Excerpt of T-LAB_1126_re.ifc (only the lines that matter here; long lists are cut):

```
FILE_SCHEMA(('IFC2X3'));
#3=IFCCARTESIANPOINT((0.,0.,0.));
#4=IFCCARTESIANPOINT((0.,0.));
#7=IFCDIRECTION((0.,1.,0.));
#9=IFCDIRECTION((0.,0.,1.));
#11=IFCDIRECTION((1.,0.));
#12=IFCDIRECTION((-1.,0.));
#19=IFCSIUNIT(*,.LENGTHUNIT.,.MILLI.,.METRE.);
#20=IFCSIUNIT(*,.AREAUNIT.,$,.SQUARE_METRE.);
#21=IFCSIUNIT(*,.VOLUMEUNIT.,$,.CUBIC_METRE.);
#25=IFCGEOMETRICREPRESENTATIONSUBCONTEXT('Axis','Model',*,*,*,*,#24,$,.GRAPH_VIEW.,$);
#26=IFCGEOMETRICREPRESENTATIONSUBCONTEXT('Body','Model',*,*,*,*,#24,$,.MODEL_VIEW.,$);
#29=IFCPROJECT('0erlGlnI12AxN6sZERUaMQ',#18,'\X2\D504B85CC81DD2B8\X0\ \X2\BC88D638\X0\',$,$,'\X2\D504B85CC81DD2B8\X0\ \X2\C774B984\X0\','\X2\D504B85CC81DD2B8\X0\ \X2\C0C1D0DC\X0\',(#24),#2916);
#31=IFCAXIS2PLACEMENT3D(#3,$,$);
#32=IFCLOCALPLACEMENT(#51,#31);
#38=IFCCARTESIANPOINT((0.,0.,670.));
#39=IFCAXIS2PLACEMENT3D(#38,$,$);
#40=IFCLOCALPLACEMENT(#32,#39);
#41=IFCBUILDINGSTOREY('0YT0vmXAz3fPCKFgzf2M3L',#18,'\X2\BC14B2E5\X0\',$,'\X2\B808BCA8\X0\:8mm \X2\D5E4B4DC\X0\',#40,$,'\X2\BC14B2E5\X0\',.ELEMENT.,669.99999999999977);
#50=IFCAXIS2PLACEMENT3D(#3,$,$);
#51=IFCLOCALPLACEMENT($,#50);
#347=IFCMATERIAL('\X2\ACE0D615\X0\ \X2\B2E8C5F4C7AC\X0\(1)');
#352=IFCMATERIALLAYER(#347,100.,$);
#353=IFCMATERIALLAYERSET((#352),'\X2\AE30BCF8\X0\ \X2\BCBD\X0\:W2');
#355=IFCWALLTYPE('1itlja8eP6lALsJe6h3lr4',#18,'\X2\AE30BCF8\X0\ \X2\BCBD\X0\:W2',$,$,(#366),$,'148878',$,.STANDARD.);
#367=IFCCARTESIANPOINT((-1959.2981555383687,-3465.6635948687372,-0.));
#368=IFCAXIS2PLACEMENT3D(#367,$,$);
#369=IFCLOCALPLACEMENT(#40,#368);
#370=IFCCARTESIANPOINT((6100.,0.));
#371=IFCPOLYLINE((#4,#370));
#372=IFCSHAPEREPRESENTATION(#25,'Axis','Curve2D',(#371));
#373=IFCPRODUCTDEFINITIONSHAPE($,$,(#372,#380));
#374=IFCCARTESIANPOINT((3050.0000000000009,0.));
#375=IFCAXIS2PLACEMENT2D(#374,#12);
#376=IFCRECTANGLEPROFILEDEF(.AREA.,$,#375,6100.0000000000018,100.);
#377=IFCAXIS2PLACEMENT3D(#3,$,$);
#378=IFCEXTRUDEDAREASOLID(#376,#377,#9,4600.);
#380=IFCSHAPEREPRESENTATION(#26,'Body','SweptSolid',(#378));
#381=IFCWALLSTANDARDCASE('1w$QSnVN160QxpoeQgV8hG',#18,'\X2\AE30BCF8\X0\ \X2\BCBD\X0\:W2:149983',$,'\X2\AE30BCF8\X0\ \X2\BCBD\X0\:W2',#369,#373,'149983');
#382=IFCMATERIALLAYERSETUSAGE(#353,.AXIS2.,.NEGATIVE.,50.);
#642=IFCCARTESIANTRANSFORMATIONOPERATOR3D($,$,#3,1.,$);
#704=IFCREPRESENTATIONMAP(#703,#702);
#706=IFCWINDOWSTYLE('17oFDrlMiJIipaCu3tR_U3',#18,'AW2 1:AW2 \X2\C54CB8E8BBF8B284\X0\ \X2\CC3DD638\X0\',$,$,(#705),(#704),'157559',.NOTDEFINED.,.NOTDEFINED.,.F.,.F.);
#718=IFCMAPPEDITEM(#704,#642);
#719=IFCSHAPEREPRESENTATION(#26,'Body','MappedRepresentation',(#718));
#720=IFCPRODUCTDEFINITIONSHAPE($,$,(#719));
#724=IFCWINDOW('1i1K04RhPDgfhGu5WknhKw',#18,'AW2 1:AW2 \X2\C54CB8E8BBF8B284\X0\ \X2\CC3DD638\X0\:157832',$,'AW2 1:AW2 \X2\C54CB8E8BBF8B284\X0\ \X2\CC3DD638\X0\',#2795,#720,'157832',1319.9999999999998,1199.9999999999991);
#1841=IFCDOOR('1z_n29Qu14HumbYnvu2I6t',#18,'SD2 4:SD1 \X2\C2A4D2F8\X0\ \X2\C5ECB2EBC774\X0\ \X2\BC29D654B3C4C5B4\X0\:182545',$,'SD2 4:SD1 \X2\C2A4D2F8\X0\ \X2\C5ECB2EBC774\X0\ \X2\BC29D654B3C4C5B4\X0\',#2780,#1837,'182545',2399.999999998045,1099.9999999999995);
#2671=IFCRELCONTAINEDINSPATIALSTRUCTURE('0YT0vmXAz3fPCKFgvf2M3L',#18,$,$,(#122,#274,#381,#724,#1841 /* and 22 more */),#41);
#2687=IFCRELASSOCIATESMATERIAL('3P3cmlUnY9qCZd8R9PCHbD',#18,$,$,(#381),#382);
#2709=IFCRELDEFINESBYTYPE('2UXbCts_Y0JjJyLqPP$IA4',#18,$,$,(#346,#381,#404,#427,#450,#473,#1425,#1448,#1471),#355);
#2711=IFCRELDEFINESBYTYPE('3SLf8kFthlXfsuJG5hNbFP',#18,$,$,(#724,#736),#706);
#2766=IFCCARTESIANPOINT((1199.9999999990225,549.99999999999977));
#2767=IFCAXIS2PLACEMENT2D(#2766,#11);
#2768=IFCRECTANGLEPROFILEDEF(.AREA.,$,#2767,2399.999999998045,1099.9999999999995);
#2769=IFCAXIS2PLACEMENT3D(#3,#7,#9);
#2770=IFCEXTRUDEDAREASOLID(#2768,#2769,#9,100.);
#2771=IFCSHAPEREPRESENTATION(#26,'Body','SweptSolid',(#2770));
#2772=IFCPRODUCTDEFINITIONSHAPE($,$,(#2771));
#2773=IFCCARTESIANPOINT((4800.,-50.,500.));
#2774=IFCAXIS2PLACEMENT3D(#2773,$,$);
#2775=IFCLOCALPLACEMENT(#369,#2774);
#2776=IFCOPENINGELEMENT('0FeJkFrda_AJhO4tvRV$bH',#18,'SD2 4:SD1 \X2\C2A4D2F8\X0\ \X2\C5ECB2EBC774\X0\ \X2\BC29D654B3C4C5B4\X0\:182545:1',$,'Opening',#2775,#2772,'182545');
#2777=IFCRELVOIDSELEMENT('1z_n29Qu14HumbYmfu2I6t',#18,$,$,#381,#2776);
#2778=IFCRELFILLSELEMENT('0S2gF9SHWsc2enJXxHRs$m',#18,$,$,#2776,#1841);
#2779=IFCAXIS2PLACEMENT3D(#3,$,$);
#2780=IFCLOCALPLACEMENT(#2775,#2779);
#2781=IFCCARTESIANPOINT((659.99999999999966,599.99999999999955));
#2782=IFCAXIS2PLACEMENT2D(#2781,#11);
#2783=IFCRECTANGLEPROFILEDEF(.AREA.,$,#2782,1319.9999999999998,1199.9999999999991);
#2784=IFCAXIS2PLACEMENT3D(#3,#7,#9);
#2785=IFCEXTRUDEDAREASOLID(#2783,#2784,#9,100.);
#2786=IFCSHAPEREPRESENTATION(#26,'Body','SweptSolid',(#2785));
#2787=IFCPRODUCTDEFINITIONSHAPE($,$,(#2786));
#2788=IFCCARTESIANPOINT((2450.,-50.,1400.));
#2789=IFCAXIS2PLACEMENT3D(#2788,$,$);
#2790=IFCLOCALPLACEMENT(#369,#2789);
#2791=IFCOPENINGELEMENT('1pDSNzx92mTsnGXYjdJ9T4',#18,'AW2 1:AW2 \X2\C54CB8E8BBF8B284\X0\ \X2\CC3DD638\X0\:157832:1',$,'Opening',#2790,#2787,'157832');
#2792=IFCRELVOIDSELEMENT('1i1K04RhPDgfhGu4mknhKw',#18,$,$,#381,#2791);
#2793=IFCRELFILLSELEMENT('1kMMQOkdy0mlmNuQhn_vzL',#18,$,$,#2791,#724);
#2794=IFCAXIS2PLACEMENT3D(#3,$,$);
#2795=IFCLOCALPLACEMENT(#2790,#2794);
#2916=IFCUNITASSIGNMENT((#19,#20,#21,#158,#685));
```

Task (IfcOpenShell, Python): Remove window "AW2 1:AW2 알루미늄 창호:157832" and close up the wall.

```python
import ifcopenshell
import ifcopenshell.api.feature
import ifcopenshell.api.root
import ifcopenshell.geom
import ifcopenshell.util.shape

model = ifcopenshell.open("T-LAB_1126_re.ifc")
settings = ifcopenshell.geom.settings()


def volume(element):
    """Net volume in cubic metres, openings subtracted."""
    shape = ifcopenshell.geom.create_shape(settings, element)
    return ifcopenshell.util.shape.get_volume(shape.geometry)


window = model.by_guid("1i1K04RhPDgfhGu5WknhKw")
opening = window.FillsVoids[0].RelatingOpeningElement
wall = opening.VoidsElements[0].RelatingBuildingElement
before = volume(wall)

ifcopenshell.api.root.remove_product(model, product=window)
ifcopenshell.api.feature.remove_feature(model, feature=opening)

after = volume(wall)

print(f"wall volume {before:.3f} -> {after:.3f} m3")

model.write("T-LAB_1126_re_v2.ifc")
```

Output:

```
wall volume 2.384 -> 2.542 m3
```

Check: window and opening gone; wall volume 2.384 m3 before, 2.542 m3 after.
